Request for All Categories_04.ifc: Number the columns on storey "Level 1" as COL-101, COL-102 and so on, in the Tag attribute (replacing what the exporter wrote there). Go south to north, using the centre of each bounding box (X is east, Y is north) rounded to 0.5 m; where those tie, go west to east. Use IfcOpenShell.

First a look at what the model holds.

```python
import ifcopenshell
import ifcopenshell.util.element
import ifcopenshell.util.placement

model = ifcopenshell.open("All Categories_04.ifc")
print(model.schema)
storey = next(s for s in model.by_type("IfcBuildingStorey") if s.Name == "Level 1")
columns = [e for e in ifcopenshell.util.element.get_decomposition(storey) if e.is_a("IfcColumn")]
for e in sorted(columns, key=lambda e: e.id()):
    origin = ifcopenshell.util.placement.get_local_placement(e.ObjectPlacement)[:3, 3]
    print(e.id(), e.Tag, e.Name, origin.round(2) + 0.0, sep=" | ")
```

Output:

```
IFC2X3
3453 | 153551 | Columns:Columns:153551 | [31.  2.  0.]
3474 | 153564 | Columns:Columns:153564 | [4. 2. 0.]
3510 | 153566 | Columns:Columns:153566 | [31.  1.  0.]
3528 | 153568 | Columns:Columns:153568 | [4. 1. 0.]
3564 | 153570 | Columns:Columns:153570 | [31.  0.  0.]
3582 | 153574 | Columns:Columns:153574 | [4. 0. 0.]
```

```python
import ifcopenshell
import ifcopenshell.geom
import ifcopenshell.util.element
import ifcopenshell.util.shape

model = ifcopenshell.open("All Categories_04.ifc")
settings = ifcopenshell.geom.settings()
settings.set("use-world-coords", True)


def centre(element):
    shape = ifcopenshell.geom.create_shape(settings, element)
    return ifcopenshell.util.shape.get_bbox_centroid(shape.geometry)


storey = next(s for s in model.by_type("IfcBuildingStorey") if s.Name == "Level 1")
columns = [e for e in ifcopenshell.util.element.get_decomposition(storey) if e.is_a("IfcColumn")]

# Insertion points can sit at a corner or the storey origin, so sort by the geometry (in metres).
centres = {e: centre(e) for e in columns}
columns.sort(key=lambda e: (round(centres[e][1] / 0.5), centres[e][0]))

for i, e in enumerate(columns, start=1):
    number = f"COL-1{i:02d}"
    e.Tag = number
    print(e.id(), number)

model.write("All Categories_04_updated.ifc")
```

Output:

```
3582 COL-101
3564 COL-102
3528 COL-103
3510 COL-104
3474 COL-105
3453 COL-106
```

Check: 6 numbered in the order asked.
